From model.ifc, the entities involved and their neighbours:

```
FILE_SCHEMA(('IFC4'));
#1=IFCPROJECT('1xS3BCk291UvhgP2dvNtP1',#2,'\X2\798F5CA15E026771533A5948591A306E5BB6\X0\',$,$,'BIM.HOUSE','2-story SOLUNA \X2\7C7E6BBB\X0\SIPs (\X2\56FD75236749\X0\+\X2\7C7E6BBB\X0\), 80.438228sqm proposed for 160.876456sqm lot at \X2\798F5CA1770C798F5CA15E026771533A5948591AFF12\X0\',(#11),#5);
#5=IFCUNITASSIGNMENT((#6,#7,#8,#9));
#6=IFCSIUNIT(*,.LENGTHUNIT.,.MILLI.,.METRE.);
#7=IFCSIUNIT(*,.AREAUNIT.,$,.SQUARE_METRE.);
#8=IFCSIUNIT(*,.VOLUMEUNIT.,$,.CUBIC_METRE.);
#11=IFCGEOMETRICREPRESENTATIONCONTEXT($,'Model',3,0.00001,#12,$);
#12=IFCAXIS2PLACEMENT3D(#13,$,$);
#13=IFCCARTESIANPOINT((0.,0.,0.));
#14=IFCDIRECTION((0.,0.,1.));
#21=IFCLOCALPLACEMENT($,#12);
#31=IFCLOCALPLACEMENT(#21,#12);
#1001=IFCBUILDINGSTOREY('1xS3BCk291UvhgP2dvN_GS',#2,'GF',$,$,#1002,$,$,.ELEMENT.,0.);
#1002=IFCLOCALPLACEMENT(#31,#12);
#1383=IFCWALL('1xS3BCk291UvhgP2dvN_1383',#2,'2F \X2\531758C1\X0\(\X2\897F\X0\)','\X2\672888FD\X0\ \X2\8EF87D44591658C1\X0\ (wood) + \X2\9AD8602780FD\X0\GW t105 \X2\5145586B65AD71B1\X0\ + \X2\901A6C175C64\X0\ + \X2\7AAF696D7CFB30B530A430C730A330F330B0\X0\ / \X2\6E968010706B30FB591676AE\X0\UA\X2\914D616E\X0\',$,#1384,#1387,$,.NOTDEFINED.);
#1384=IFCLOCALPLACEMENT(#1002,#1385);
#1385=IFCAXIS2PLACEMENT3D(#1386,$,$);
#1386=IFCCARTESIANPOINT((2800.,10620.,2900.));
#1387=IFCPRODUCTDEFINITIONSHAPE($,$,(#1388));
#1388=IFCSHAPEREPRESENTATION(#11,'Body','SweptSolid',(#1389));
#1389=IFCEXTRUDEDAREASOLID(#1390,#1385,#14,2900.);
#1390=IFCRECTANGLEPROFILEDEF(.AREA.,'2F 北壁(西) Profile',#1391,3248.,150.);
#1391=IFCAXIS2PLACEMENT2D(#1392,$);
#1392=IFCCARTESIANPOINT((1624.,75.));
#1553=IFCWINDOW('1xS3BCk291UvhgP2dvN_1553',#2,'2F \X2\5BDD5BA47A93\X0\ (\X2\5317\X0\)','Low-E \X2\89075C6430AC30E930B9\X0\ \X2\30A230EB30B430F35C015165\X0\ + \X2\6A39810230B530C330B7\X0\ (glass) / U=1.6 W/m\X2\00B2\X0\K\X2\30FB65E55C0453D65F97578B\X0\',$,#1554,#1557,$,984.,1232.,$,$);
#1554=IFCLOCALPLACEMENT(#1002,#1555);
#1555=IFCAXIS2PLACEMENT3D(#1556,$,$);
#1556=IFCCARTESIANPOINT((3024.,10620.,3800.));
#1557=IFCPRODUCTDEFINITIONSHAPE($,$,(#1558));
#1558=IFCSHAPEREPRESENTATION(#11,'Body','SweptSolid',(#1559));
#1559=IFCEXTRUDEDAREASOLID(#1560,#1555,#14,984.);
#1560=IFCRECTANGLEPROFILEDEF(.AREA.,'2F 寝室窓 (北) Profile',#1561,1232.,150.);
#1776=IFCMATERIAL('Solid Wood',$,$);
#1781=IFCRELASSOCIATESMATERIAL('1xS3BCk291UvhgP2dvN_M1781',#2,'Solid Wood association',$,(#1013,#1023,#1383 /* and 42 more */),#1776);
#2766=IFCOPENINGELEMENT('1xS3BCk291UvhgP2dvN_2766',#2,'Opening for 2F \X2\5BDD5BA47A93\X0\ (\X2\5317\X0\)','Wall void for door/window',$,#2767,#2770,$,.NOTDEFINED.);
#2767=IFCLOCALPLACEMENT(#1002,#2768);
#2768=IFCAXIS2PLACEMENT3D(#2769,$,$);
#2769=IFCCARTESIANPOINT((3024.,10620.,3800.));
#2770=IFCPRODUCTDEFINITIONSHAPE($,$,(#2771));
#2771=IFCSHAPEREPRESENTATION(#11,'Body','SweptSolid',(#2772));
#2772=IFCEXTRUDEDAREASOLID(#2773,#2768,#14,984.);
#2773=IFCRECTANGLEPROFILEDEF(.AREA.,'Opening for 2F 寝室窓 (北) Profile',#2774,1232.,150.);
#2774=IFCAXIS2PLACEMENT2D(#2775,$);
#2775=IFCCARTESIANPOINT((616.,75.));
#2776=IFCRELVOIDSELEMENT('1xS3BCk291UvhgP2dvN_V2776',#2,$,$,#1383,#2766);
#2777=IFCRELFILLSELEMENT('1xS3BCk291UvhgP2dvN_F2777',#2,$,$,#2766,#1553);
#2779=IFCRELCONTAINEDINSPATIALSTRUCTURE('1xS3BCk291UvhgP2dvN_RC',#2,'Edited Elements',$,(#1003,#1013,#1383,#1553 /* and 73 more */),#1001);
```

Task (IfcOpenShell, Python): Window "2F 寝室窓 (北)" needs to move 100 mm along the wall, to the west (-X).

```python
import ifcopenshell
import ifcopenshell.api.geometry
import ifcopenshell.util.placement

model = ifcopenshell.open("model.ifc")

window = model.by_guid("1xS3BCk291UvhgP2dvN_1553")
opening = window.FillsVoids[0].RelatingOpeningElement
wall = opening.VoidsElements[0].RelatingBuildingElement

wall_matrix = ifcopenshell.util.placement.get_local_placement(wall.ObjectPlacement)
shift = wall_matrix[:3, 0] * -100.0
before = ifcopenshell.util.placement.get_local_placement(window.ObjectPlacement)[:3, 3].copy()

# The window is not placed relative to its opening, so move both.
for product in (opening, window):
    matrix = ifcopenshell.util.placement.get_local_placement(product.ObjectPlacement)
    matrix[:3, 3] += shift
    ifcopenshell.api.geometry.edit_object_placement(model, product=product, matrix=matrix, is_si=False)

after = ifcopenshell.util.placement.get_local_placement(window.ObjectPlacement)[:3, 3]
print("window moved by", (after - before).round(3) + 0.0)

model.write("model_updated.ifc")
```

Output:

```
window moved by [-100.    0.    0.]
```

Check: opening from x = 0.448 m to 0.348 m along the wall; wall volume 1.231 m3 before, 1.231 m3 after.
